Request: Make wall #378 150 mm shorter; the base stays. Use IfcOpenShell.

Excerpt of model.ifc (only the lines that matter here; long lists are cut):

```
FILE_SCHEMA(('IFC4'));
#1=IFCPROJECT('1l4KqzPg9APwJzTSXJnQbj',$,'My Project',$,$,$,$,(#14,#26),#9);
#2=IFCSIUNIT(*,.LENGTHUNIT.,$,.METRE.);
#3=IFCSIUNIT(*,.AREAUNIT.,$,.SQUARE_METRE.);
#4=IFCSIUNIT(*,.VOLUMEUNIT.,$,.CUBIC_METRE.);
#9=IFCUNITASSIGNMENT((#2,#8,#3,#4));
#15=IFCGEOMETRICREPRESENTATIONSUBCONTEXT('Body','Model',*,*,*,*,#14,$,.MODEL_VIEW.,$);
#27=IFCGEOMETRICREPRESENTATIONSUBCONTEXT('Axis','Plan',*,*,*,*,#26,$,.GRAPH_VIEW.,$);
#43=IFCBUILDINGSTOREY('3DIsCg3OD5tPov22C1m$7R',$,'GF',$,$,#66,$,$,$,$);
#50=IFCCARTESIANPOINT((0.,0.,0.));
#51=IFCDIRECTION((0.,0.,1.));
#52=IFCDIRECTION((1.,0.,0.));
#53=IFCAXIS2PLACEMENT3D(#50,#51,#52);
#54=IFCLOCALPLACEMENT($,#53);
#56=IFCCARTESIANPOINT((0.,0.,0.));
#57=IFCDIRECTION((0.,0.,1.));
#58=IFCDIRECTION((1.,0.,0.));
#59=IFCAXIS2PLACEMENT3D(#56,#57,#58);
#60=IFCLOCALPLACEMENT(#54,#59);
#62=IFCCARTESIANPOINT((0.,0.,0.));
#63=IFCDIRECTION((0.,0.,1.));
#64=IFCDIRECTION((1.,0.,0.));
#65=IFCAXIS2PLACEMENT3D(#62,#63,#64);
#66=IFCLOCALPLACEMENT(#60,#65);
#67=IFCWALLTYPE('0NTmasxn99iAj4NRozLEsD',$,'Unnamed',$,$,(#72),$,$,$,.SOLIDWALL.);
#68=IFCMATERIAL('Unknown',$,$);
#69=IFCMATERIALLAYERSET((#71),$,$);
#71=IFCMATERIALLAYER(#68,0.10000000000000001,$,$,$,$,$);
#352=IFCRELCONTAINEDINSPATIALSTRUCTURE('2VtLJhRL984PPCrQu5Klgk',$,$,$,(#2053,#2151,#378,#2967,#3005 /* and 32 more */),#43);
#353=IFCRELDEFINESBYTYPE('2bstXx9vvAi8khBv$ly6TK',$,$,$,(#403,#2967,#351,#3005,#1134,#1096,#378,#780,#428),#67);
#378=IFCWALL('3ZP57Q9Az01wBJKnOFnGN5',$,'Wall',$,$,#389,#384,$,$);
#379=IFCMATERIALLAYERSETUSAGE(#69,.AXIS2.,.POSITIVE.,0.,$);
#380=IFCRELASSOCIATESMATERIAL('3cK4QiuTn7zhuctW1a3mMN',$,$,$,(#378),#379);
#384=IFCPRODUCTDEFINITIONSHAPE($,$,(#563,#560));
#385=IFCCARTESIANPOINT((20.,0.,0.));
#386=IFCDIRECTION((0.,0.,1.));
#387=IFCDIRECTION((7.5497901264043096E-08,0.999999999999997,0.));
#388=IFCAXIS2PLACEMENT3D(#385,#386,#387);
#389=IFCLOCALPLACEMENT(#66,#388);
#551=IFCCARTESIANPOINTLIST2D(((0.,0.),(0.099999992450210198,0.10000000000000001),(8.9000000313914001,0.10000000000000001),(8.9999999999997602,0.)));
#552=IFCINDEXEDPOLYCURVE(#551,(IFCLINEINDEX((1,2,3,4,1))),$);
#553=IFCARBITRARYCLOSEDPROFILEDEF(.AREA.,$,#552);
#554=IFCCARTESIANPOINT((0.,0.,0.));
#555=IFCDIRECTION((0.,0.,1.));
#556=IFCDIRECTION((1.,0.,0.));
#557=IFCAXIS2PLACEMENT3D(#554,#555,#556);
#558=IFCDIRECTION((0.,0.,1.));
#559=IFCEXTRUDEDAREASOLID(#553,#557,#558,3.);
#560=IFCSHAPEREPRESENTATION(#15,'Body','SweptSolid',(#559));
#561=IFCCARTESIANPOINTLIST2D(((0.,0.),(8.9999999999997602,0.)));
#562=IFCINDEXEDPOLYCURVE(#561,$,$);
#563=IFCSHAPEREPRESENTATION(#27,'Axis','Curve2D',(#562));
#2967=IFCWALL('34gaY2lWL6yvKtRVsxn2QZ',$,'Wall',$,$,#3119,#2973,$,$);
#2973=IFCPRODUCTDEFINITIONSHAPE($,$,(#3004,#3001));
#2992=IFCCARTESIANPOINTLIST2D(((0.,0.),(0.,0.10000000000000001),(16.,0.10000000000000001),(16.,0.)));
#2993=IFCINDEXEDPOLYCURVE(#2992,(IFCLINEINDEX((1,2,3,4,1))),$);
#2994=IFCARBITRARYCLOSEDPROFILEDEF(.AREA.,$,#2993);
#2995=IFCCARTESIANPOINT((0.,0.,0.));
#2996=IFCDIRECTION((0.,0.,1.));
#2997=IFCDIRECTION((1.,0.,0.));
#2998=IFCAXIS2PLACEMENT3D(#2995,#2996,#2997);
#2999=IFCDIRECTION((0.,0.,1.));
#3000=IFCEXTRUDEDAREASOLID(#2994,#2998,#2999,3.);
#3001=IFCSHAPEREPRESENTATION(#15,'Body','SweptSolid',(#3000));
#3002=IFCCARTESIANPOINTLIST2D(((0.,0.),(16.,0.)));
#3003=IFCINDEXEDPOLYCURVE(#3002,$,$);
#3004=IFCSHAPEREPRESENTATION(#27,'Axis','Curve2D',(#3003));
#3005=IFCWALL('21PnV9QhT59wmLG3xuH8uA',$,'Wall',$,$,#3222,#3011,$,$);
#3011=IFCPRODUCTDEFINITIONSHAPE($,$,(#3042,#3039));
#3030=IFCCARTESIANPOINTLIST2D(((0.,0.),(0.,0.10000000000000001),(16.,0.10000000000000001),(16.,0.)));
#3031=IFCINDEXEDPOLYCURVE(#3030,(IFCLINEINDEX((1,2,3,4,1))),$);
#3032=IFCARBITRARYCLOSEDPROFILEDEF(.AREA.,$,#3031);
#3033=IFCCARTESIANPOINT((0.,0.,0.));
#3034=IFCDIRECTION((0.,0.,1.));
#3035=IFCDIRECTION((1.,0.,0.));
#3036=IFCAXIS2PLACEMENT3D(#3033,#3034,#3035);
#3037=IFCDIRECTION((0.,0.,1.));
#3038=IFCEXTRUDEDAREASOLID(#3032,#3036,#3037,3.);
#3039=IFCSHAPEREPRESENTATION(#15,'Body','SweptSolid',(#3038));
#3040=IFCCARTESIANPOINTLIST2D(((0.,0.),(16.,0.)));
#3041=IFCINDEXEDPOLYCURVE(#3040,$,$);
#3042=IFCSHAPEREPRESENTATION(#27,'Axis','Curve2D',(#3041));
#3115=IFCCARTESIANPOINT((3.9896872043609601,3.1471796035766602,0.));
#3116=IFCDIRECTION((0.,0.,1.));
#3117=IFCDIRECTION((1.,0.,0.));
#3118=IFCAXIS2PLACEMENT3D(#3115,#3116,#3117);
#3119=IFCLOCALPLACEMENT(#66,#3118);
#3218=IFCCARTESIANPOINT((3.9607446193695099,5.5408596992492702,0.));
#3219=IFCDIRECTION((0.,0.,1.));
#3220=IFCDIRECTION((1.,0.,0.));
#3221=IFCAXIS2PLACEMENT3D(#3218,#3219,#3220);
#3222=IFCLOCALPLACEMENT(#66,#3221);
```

```python
import ifcopenshell
import ifcopenshell.geom
import ifcopenshell.util.representation
import ifcopenshell.util.shape
import ifcopenshell.util.unit

model = ifcopenshell.open("model.ifc")
unit_scale = ifcopenshell.util.unit.calculate_unit_scale(model)
settings = ifcopenshell.geom.settings()


def volume(element):
    """Net volume in cubic metres, openings subtracted."""
    shape = ifcopenshell.geom.create_shape(settings, element)
    return ifcopenshell.util.shape.get_volume(shape.geometry)


wall = model.by_id(378)
before = volume(wall)

body = ifcopenshell.util.representation.get_representation(wall, "Model", "Body")
solid = body.Items[0]
old_height = solid.Depth
solid.Depth -= 0.15 / unit_scale
after = volume(wall)

print(f"height {old_height:g} -> {solid.Depth:g}, volume {before:.3f} -> {after:.3f} m3")

model.write("model_updated.ifc")
```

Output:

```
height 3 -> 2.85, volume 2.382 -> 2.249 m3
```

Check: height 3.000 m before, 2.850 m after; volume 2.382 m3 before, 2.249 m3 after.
